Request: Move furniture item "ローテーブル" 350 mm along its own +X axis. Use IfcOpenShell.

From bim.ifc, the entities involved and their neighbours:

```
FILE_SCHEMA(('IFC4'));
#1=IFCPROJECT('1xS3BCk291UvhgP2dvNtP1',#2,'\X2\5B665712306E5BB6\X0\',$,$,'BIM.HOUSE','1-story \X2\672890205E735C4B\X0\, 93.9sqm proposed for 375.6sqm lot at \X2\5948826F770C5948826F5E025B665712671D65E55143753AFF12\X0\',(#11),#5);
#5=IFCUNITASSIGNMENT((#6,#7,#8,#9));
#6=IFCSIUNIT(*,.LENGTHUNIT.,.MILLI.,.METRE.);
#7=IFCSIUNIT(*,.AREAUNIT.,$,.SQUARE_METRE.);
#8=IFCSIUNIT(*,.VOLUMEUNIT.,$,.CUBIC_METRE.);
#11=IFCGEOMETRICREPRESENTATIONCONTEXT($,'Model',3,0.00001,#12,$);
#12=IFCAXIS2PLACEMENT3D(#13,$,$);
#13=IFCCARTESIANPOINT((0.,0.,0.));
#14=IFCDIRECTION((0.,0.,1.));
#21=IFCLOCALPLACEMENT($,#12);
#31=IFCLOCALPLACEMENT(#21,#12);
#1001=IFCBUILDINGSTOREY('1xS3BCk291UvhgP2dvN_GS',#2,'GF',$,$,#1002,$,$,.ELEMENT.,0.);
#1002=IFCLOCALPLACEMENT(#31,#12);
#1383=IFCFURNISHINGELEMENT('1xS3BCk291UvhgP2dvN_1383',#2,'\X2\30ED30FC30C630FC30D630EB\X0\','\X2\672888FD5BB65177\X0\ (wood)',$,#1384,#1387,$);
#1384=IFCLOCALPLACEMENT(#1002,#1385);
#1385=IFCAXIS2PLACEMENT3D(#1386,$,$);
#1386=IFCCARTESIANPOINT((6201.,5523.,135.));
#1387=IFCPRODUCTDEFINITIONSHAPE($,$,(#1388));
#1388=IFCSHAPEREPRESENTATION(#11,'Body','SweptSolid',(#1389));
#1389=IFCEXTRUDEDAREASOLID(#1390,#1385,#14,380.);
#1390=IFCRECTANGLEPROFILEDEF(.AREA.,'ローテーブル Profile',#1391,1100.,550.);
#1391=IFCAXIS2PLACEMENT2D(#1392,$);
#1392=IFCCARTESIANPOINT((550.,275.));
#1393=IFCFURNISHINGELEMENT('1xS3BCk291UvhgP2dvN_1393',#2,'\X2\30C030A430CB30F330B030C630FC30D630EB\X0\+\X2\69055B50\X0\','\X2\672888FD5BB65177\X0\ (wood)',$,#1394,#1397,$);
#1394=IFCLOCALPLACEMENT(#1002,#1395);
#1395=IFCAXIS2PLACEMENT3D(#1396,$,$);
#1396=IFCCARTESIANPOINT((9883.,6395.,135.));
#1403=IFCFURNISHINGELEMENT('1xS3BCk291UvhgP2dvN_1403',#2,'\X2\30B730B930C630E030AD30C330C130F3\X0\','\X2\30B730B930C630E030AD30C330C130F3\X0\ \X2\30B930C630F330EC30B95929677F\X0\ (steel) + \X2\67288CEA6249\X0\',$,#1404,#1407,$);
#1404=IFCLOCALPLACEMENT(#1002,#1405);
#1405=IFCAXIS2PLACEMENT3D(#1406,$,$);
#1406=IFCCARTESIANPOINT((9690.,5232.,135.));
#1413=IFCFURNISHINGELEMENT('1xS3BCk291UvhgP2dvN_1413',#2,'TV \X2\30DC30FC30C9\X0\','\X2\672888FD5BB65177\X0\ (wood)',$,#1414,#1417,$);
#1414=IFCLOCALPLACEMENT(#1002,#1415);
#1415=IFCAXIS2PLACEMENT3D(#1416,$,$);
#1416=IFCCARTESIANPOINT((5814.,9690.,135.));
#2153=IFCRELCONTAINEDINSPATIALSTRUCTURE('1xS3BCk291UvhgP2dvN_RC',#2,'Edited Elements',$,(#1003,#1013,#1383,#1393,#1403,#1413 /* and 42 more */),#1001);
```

```python
import ifcopenshell
import ifcopenshell.api.geometry
import ifcopenshell.util.placement

model = ifcopenshell.open("bim.ifc")

item = model.by_guid("1xS3BCk291UvhgP2dvN_1383")
matrix = ifcopenshell.util.placement.get_local_placement(item.ObjectPlacement)
matrix[:3, 3] += matrix[:3, 0] * 350.0
ifcopenshell.api.geometry.edit_object_placement(model, product=item, matrix=matrix, is_si=False)

print(ifcopenshell.util.placement.get_local_placement(item.ObjectPlacement).round(3) + 0.0)

model.write("bim_v2.ifc")
```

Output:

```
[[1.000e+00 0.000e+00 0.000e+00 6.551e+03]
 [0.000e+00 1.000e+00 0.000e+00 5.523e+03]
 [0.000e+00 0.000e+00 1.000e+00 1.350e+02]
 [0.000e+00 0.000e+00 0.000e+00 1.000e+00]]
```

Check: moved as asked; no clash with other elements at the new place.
